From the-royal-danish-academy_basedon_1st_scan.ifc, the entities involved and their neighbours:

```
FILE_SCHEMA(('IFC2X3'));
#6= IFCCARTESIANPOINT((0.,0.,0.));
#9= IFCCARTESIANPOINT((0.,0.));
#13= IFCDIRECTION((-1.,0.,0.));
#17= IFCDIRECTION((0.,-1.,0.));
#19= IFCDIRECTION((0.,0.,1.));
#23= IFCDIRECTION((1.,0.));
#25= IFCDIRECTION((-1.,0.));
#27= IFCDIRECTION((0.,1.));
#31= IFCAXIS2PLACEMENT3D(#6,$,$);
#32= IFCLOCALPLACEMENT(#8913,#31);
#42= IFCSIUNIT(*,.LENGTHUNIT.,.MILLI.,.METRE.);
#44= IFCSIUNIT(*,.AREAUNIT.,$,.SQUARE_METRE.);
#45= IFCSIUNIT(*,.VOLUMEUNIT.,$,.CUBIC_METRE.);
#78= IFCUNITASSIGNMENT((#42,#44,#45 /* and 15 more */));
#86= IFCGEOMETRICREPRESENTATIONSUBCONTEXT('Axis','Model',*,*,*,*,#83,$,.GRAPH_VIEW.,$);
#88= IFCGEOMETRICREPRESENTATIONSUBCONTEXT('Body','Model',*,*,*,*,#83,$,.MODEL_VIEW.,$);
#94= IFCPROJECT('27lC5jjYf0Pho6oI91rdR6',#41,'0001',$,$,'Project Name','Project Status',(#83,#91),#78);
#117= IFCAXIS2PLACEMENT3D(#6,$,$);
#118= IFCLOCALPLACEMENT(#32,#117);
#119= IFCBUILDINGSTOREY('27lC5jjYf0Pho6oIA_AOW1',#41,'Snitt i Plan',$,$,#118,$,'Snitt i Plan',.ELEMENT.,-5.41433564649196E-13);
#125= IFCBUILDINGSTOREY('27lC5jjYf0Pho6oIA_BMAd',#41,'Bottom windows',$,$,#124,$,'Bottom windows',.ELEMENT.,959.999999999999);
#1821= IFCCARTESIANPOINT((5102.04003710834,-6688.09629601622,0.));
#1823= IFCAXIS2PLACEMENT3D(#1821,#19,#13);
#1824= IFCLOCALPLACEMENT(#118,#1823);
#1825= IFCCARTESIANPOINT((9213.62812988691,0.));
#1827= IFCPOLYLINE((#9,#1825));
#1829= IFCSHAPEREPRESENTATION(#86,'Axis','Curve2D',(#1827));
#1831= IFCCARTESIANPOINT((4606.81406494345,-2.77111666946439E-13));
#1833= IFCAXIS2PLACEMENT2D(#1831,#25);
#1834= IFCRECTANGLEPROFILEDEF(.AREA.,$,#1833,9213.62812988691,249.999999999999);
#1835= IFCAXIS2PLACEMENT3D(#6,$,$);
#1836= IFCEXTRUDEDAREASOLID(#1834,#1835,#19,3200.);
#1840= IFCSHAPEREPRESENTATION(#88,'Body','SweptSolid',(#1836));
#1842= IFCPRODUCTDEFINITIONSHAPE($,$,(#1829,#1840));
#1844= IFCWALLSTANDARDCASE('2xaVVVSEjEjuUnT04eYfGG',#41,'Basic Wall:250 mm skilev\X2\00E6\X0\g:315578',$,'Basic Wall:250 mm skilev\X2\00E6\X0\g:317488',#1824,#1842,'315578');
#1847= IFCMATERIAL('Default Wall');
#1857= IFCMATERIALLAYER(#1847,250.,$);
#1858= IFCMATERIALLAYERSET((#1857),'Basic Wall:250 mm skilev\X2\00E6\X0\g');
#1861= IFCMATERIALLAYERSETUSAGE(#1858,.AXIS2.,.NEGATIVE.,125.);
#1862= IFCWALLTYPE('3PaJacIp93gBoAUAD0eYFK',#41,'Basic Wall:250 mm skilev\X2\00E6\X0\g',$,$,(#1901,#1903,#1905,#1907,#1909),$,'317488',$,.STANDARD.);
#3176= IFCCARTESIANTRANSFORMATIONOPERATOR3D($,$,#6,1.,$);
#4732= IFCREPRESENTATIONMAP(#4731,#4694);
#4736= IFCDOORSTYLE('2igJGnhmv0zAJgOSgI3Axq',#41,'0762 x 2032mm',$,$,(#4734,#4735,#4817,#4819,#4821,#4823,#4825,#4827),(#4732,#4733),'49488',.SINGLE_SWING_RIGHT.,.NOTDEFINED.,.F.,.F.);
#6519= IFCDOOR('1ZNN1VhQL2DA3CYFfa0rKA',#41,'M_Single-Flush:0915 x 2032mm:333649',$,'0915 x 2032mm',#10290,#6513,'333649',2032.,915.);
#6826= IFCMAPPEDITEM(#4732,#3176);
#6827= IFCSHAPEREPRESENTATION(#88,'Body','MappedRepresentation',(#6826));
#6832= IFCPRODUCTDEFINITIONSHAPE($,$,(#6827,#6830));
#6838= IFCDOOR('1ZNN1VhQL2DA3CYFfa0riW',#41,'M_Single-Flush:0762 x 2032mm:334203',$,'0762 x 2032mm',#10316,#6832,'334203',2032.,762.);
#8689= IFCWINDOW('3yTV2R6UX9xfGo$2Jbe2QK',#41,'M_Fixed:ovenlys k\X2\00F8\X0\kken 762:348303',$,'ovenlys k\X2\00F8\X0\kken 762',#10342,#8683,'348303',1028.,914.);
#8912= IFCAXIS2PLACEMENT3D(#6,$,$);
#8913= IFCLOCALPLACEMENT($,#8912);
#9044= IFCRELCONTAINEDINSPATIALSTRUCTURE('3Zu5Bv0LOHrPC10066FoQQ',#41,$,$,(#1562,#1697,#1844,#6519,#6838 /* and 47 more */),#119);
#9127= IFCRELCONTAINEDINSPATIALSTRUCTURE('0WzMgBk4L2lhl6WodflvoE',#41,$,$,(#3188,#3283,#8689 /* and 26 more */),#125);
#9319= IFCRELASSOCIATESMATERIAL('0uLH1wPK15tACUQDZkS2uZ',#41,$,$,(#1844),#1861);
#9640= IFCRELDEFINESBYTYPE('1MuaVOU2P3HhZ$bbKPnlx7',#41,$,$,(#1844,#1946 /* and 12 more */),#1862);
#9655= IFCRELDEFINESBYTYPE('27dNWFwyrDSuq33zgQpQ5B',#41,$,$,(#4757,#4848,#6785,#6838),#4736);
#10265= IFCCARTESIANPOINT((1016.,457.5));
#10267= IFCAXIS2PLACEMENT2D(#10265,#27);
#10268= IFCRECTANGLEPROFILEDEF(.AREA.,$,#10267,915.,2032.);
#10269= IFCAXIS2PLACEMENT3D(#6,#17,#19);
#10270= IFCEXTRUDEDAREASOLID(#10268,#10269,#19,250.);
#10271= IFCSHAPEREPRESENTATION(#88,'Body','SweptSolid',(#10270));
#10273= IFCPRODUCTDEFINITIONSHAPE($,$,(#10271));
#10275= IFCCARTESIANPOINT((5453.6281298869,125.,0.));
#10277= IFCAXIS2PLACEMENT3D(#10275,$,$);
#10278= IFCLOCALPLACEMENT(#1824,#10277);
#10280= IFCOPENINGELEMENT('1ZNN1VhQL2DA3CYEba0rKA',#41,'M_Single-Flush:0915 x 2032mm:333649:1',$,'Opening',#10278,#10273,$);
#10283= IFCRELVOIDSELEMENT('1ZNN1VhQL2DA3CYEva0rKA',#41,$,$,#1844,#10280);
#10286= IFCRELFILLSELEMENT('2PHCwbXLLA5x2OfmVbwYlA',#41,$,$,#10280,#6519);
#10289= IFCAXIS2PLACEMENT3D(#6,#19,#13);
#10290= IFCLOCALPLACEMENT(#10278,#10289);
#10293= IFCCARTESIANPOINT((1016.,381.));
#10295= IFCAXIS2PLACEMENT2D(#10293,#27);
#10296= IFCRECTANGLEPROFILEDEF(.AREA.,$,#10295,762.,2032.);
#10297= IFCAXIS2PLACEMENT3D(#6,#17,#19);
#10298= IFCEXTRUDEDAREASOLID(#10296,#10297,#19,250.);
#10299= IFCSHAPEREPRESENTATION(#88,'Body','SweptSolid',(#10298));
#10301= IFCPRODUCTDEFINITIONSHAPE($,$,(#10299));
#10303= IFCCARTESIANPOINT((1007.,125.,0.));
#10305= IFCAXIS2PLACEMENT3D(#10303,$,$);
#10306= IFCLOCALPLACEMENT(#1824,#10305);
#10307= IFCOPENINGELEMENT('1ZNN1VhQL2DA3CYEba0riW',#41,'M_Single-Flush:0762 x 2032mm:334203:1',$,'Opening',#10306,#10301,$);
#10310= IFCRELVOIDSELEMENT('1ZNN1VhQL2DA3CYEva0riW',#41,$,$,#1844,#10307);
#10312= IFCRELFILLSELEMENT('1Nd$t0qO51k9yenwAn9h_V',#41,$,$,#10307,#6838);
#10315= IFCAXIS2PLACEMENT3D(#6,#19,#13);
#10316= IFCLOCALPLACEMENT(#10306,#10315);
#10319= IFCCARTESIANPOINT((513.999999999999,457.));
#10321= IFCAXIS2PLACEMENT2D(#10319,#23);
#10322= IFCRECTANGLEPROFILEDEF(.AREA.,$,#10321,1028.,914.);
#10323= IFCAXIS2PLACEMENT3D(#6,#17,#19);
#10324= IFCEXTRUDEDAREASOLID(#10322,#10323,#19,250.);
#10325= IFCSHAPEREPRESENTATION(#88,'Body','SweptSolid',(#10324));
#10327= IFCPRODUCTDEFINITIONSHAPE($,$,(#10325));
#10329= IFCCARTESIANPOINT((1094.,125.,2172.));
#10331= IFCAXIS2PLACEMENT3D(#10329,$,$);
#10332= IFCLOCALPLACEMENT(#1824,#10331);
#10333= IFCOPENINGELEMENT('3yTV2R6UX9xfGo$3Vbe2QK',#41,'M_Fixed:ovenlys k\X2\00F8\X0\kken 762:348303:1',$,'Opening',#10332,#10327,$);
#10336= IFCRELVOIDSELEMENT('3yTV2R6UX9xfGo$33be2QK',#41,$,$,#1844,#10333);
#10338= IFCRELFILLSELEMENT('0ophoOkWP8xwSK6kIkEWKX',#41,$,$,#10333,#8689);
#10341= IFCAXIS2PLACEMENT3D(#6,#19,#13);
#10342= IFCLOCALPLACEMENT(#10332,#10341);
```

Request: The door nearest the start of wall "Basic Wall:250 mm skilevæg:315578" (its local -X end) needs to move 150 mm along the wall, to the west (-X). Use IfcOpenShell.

```python
import ifcopenshell
import ifcopenshell.api.geometry
import ifcopenshell.util.placement
import ifcopenshell.util.unit

model = ifcopenshell.open("the-royal-danish-academy_basedon_1st_scan.ifc")
unit_scale = ifcopenshell.util.unit.calculate_unit_scale(model)

door = model.by_guid("1ZNN1VhQL2DA3CYFfa0riW")
opening = door.FillsVoids[0].RelatingOpeningElement
wall = opening.VoidsElements[0].RelatingBuildingElement

wall_matrix = ifcopenshell.util.placement.get_local_placement(wall.ObjectPlacement)
shift = wall_matrix[:3, 0] * 0.15 / unit_scale
before = ifcopenshell.util.placement.get_local_placement(door.ObjectPlacement)[:3, 3].copy()

# The door is placed relative to its opening, so it follows when the opening moves.
matrix = ifcopenshell.util.placement.get_local_placement(opening.ObjectPlacement)
matrix[:3, 3] += shift
ifcopenshell.api.geometry.edit_object_placement(
    model, product=opening, matrix=matrix, is_si=False, should_transform_children=True
)

after = ifcopenshell.util.placement.get_local_placement(door.ObjectPlacement)[:3, 3]
print("door moved by", (after - before).round(3) + 0.0)

model.write("the-royal-danish-academy_basedon_1st_scan_v2.ifc")
```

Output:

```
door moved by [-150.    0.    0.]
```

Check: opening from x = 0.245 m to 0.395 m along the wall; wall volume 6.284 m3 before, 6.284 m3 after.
